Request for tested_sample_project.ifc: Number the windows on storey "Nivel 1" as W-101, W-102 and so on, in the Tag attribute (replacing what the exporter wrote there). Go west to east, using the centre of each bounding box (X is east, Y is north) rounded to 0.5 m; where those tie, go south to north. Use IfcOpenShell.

First a look at what the model holds.

```python
import ifcopenshell
import ifcopenshell.util.element
import ifcopenshell.util.placement

model = ifcopenshell.open("tested_sample_project.ifc")
print(model.schema)
storey = next(s for s in model.by_type("IfcBuildingStorey") if s.Name == "Nivel 1")
windows = [e for e in ifcopenshell.util.element.get_decomposition(storey) if e.is_a("IfcWindow")]
for e in sorted(windows, key=lambda e: e.id()):
    origin = ifcopenshell.util.placement.get_local_placement(e.ObjectPlacement)[:3, 3]
    print(e.id(), e.Tag, e.Name, origin.round(2) + 0.0, sep=" | ")
```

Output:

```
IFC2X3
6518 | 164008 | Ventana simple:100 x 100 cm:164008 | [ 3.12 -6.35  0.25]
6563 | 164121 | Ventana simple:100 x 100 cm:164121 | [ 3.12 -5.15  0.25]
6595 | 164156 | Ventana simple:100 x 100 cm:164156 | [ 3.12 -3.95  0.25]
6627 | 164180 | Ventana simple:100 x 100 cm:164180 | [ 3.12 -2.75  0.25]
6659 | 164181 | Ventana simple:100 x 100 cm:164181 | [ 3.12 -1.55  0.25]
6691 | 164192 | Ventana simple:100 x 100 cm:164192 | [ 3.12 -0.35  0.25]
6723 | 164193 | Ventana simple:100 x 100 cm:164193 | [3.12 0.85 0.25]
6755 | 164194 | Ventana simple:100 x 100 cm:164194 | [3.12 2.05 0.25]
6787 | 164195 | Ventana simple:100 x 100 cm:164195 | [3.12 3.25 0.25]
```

```python
import ifcopenshell
import ifcopenshell.geom
import ifcopenshell.util.element
import ifcopenshell.util.shape

model = ifcopenshell.open("tested_sample_project.ifc")
settings = ifcopenshell.geom.settings()
settings.set("use-world-coords", True)


def centre(element):
    shape = ifcopenshell.geom.create_shape(settings, element)
    return ifcopenshell.util.shape.get_bbox_centroid(shape.geometry)


storey = next(s for s in model.by_type("IfcBuildingStorey") if s.Name == "Nivel 1")
windows = [e for e in ifcopenshell.util.element.get_decomposition(storey) if e.is_a("IfcWindow")]

# Insertion points can sit at a corner or the storey origin, so sort by the geometry (in metres).
centres = {e: centre(e) for e in windows}
windows.sort(key=lambda e: (round(centres[e][0] / 0.5), centres[e][1]))

for i, e in enumerate(windows, start=1):
    number = f"W-1{i:02d}"
    e.Tag = number
    print(e.id(), number)

model.write("tested_sample_project_v2.ifc")
```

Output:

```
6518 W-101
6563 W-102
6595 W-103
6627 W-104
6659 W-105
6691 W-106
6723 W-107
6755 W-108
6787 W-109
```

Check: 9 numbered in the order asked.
